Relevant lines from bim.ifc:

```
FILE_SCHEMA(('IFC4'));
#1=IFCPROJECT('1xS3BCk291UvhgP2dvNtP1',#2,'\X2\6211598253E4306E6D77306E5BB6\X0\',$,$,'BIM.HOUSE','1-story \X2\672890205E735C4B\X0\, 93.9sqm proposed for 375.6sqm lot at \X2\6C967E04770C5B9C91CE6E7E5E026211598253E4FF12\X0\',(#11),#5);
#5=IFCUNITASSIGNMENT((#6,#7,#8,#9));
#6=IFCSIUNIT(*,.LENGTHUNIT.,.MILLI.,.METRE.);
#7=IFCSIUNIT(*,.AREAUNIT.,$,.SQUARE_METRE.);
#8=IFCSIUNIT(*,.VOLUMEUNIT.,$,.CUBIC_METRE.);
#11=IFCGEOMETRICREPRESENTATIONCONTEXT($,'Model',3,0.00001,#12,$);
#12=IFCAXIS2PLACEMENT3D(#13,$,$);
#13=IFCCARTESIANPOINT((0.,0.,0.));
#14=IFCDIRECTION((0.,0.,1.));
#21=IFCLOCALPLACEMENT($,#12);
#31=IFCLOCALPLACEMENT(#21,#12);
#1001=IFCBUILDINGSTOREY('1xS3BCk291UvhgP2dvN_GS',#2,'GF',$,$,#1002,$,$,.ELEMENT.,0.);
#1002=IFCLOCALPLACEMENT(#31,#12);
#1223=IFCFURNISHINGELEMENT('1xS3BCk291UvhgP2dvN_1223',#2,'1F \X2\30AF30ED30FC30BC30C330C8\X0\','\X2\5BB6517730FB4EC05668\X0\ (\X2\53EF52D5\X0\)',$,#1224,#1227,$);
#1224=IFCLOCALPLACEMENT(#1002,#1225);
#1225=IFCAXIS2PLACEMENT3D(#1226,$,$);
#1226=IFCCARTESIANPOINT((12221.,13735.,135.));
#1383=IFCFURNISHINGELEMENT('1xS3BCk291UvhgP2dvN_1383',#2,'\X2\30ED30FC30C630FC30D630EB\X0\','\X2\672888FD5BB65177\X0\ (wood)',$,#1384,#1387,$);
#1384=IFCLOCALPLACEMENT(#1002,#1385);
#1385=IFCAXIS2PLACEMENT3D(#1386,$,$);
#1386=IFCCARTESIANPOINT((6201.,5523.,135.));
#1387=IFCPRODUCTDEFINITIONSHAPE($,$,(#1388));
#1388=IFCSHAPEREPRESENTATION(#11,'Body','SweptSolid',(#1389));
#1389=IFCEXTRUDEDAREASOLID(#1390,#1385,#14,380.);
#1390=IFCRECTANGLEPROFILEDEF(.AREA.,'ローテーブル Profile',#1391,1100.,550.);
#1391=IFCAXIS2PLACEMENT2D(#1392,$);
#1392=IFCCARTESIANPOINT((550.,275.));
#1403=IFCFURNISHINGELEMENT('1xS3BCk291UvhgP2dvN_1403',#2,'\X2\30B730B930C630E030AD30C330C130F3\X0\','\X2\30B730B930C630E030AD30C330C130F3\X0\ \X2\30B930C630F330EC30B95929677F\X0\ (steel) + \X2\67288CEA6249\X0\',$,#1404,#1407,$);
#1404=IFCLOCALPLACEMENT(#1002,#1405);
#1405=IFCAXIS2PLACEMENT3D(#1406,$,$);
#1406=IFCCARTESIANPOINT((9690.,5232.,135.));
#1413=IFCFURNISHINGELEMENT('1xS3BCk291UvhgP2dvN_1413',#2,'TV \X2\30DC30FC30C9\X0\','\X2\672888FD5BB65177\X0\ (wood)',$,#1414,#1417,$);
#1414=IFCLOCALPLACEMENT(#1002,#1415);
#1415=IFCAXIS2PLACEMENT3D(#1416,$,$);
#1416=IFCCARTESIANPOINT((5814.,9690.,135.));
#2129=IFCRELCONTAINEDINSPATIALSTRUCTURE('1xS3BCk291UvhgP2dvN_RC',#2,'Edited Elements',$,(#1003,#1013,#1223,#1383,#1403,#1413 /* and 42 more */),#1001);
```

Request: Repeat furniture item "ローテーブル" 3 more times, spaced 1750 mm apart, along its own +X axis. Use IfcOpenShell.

```python
import ifcopenshell
import ifcopenshell.api.geometry
import ifcopenshell.api.root
import ifcopenshell.util.element
import ifcopenshell.util.placement
import ifcopenshell.util.unit

model = ifcopenshell.open("bim.ifc")
unit_scale = ifcopenshell.util.unit.calculate_unit_scale(model)


def reuse_history(source, copy):
    """copy_class also copies each property set's owner history, people and application; keep the originals."""
    for rel in copy.IsDefinedBy:
        if rel.is_a("IfcRelDefinesByProperties") and (history := rel.RelatingPropertyDefinition.OwnerHistory):
            rel.RelatingPropertyDefinition.OwnerHistory = source.OwnerHistory
            ifcopenshell.util.element.remove_deep2(model, history)


source = model.by_id(1383)
base = ifcopenshell.util.placement.get_local_placement(source.ObjectPlacement)
step = base[:3, 0] * 1.75 / unit_scale

for i in range(1, 4):
    copy = ifcopenshell.api.root.copy_class(model, product=source)
    copy.Representation = ifcopenshell.util.element.copy_deep(
        model, source.Representation, exclude=["IfcGeometricRepresentationContext", "IfcRepresentationMap"]
    )
    reuse_history(source, copy)
    matrix = base.copy()
    matrix[:3, 3] += i * step
    print("added at", matrix[:3, 3].round(3) + 0.0)
    ifcopenshell.api.geometry.edit_object_placement(model, product=copy, matrix=matrix, is_si=False)

model.write("bim_rev.ifc")
```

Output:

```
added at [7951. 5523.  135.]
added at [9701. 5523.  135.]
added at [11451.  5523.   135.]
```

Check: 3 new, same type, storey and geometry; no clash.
